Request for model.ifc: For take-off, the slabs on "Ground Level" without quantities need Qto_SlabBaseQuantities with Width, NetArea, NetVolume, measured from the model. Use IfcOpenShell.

First a look at what the model holds.

```python
import ifcopenshell
import ifcopenshell.util.element
import ifcopenshell.util.unit

model = ifcopenshell.open("model.ifc")
print(model.schema)
for unit_type in ("LENGTHUNIT", "AREAUNIT", "VOLUMEUNIT"):
    print(unit_type, ifcopenshell.util.unit.calculate_unit_scale(model, unit_type))
storey = next(s for s in model.by_type("IfcBuildingStorey") if s.Name == "Ground Level")
slabs = [e for e in ifcopenshell.util.element.get_decomposition(storey) if e.is_a("IfcSlab")]
for e in sorted(slabs, key=lambda e: e.id()):
    print(e.id(), e.is_a(), e.Name, list(ifcopenshell.util.element.get_psets(e, qtos_only=True)), sep=" | ")
```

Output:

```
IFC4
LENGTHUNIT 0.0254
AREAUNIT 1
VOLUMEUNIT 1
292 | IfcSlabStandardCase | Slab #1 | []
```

```python
import ifcopenshell
import ifcopenshell.api.pset
import ifcopenshell.geom
import ifcopenshell.util.element
import ifcopenshell.util.shape
import ifcopenshell.util.unit

model = ifcopenshell.open("model.ifc")
unit_scale = ifcopenshell.util.unit.calculate_unit_scale(model)
area_scale = ifcopenshell.util.unit.calculate_unit_scale(model, "AREAUNIT")
volume_scale = ifcopenshell.util.unit.calculate_unit_scale(model, "VOLUMEUNIT")
settings = ifcopenshell.geom.settings()

storey = next(s for s in model.by_type("IfcBuildingStorey") if s.Name == "Ground Level")
slabs = [e for e in ifcopenshell.util.element.get_decomposition(storey) if e.is_a("IfcSlab")]

for e in sorted(slabs, key=lambda e: e.id()):
    if ifcopenshell.util.element.get_psets(e, qtos_only=True, should_inherit=False):
        continue
    # Geometry comes back in metres, in the element's own axes.
    shape = ifcopenshell.geom.create_shape(settings, e)
    values = {
        "Width": ifcopenshell.util.shape.get_z(shape.geometry) / unit_scale,
        "NetArea": ifcopenshell.util.shape.get_footprint_area(shape.geometry) / area_scale,
        "NetVolume": ifcopenshell.util.shape.get_volume(shape.geometry) / volume_scale,
    }
    qto = ifcopenshell.api.pset.add_qto(model, product=e, name="Qto_SlabBaseQuantities")
    ifcopenshell.api.pset.edit_qto(model, qto=qto, properties=values)
    print(e.id(), {k: round(v, 3) for k, v in values.items()})

model.write("model_v2.ifc")
```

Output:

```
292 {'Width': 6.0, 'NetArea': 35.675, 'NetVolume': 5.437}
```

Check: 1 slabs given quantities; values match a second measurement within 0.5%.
